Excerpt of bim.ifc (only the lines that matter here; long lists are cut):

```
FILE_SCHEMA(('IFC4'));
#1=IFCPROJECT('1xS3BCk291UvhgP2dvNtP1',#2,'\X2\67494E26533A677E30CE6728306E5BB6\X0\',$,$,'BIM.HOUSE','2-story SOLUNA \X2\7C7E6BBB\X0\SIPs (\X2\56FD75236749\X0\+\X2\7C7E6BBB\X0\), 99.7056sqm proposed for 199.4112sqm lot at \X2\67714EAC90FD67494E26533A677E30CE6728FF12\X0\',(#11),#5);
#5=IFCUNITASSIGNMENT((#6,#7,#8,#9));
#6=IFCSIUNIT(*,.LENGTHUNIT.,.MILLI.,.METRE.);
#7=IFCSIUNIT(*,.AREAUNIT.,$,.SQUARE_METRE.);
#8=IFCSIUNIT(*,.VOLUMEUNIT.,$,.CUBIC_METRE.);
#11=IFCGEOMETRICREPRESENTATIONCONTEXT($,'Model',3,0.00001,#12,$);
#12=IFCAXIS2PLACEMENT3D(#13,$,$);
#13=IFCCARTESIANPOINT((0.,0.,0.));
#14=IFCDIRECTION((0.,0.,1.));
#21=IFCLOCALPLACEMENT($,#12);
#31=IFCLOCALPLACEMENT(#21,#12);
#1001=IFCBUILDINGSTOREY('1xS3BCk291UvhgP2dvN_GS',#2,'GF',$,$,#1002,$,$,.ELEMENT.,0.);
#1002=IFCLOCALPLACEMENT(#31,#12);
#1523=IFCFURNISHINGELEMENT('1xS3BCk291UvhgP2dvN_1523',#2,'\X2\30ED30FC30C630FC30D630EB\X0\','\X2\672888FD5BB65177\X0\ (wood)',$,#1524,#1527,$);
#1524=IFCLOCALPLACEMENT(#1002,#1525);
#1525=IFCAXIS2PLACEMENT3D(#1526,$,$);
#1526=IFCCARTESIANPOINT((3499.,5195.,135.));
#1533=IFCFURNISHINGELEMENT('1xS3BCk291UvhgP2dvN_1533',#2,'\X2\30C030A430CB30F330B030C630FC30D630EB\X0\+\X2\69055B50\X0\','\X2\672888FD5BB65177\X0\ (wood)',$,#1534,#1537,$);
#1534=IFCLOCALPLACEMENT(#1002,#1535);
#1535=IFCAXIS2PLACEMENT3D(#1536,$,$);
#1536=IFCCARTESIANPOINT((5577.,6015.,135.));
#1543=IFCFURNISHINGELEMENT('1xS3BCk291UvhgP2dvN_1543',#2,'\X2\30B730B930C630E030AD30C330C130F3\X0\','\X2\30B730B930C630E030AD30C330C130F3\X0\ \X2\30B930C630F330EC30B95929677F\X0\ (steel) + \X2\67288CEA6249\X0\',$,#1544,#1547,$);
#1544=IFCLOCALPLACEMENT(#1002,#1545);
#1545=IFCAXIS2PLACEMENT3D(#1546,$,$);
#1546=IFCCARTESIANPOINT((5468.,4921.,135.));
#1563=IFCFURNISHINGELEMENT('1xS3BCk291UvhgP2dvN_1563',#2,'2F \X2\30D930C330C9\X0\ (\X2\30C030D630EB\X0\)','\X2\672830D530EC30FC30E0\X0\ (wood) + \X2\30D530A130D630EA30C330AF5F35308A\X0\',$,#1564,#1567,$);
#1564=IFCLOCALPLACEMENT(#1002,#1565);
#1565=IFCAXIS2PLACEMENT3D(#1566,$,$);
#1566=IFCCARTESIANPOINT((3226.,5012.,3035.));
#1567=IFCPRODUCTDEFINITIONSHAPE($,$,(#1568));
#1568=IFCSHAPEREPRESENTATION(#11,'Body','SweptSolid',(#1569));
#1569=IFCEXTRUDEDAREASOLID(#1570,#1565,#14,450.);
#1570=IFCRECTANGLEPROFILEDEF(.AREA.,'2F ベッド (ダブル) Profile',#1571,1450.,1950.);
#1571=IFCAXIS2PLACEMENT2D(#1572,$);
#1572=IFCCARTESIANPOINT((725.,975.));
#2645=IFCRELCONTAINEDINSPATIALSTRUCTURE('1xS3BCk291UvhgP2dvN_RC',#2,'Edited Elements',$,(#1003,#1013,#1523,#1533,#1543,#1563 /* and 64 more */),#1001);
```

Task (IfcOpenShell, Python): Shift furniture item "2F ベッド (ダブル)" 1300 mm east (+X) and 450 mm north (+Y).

```python
import ifcopenshell
import ifcopenshell.api.geometry
import ifcopenshell.util.placement
import ifcopenshell.util.unit

model = ifcopenshell.open("bim.ifc")
unit_scale = ifcopenshell.util.unit.calculate_unit_scale(model)

item = model.by_guid("1xS3BCk291UvhgP2dvN_1563")
matrix = ifcopenshell.util.placement.get_local_placement(item.ObjectPlacement)
matrix[0, 3] += 1.3 / unit_scale
matrix[1, 3] += 0.45 / unit_scale
ifcopenshell.api.geometry.edit_object_placement(model, product=item, matrix=matrix, is_si=False)

print(ifcopenshell.util.placement.get_local_placement(item.ObjectPlacement).round(3) + 0.0)

model.write("bim_rev.ifc")
```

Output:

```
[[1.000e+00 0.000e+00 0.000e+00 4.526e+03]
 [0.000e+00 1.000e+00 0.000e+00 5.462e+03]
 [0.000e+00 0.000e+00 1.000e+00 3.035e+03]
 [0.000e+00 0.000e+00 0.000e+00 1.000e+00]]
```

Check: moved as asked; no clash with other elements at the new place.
